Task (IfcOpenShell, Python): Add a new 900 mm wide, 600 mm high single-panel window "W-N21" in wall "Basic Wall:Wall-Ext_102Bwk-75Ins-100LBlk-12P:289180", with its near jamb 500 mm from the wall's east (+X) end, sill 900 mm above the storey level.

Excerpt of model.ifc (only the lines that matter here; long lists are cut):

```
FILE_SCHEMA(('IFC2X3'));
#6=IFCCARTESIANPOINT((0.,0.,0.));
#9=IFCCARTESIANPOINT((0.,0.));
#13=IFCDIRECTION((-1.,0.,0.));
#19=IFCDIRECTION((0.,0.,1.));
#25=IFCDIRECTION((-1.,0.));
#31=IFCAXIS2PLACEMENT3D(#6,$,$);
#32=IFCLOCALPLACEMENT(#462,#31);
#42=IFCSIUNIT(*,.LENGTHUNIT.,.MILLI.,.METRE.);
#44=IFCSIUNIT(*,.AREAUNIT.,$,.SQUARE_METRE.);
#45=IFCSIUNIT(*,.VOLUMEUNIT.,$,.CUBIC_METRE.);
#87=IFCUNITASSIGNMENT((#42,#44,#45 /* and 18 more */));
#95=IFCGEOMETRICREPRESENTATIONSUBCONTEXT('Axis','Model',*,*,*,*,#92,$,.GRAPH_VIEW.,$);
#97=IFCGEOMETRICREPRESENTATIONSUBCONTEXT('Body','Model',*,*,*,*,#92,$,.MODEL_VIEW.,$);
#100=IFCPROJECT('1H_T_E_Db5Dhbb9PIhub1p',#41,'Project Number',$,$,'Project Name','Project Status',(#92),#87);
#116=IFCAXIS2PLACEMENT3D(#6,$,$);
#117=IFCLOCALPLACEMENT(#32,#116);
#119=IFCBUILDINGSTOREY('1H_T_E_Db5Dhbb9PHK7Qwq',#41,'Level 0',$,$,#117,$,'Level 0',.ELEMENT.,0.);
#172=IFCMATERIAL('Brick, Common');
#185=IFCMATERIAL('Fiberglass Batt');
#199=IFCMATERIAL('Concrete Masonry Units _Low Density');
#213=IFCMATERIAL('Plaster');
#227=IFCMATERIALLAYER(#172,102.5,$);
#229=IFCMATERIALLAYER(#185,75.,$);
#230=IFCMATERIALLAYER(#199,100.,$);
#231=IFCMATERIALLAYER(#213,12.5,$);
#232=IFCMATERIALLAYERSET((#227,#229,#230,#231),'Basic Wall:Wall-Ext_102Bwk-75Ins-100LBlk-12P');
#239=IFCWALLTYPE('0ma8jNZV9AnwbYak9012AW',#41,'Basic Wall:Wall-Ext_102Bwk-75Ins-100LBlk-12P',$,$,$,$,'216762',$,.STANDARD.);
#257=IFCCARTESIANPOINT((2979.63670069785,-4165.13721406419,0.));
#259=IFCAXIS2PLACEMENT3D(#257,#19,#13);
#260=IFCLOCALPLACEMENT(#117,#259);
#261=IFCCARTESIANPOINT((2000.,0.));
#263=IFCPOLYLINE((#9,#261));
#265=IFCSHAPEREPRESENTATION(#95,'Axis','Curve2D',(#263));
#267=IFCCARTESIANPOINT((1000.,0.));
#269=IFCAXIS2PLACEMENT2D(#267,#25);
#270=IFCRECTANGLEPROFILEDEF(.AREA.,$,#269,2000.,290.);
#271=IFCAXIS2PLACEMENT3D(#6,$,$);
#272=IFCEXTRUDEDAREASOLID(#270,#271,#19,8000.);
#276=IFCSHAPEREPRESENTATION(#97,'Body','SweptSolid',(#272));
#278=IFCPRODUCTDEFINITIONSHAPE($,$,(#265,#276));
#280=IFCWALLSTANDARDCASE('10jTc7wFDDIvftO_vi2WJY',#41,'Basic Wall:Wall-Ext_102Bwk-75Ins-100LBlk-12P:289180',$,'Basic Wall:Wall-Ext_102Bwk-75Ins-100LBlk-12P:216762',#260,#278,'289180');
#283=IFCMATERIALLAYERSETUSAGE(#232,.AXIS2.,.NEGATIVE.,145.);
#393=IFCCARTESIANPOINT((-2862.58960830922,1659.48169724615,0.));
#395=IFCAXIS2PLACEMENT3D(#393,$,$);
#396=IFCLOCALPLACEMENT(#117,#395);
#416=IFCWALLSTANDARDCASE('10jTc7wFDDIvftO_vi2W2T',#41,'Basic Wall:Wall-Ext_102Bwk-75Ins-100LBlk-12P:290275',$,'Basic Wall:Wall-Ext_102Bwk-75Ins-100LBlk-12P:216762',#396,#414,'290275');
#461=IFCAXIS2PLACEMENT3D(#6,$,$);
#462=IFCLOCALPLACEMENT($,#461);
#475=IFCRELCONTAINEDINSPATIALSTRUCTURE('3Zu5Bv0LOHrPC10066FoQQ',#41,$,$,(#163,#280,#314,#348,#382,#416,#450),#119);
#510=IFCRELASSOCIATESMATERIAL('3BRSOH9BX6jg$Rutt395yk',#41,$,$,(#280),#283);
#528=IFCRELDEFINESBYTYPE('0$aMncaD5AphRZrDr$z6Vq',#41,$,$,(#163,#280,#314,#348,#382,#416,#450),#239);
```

```python
import numpy as np
import ifcopenshell
import ifcopenshell.api.feature
import ifcopenshell.api.geometry
import ifcopenshell.api.root
import ifcopenshell.api.spatial
import ifcopenshell.api.type
import ifcopenshell.geom
import ifcopenshell.util.element
import ifcopenshell.util.placement
import ifcopenshell.util.representation
import ifcopenshell.util.shape
import ifcopenshell.util.unit

model = ifcopenshell.open("model.ifc")
unit_scale = ifcopenshell.util.unit.calculate_unit_scale(model)
settings = ifcopenshell.geom.settings()


def volume(element):
    """Net volume in cubic metres, openings subtracted."""
    shape = ifcopenshell.geom.create_shape(settings, element)
    return ifcopenshell.util.shape.get_volume(shape.geometry)


wall = model.by_guid("10jTc7wFDDIvftO_vi2WJY")
storey = ifcopenshell.util.element.get_container(wall, ifc_class="IfcBuildingStorey")
context = ifcopenshell.util.representation.get_context(model, "Model", "Body", "MODEL_VIEW")
before = volume(wall)

width, height, from_end, sill = 0.9, 0.6, 0.5, 0.9  # metres

# The wall runs along its own X axis, and the end named is its -X end.
wall_shape = ifcopenshell.geom.create_shape(settings, wall)
x, y, z = ifcopenshell.util.shape.get_vertices(wall_shape.geometry).T
start = x.min() + from_end
face, thickness = float(y.min()), float(y.max() - y.min())
wall_matrix = ifcopenshell.util.placement.get_local_placement(wall.ObjectPlacement)
level = ifcopenshell.util.placement.get_local_placement(storey.ObjectPlacement)[2, 3]


def in_wall(x, y):
    """Placement at x, y metres in the wall's axes, at sill height."""
    matrix = wall_matrix.copy()
    matrix[:, 3] = wall_matrix @ np.array([x / unit_scale, y / unit_scale, 0.0, 1.0])
    matrix[2, 3] = level + sill / unit_scale
    return matrix


# Opening: a box that overshoots both wall faces by 50 mm.
opening = ifcopenshell.api.root.create_entity(model, ifc_class="IfcOpeningElement")
box = ifcopenshell.api.geometry.add_wall_representation(
    model, context=context, length=width, height=height, thickness=thickness + 0.1
)
ifcopenshell.api.geometry.assign_representation(model, product=opening, representation=box)
ifcopenshell.api.geometry.edit_object_placement(model, product=opening, matrix=in_wall(start, face - 0.05), is_si=False)
ifcopenshell.api.feature.add_feature(model, feature=opening, element=wall)

window = ifcopenshell.api.root.create_entity(model, ifc_class="IfcWindow", name="W-N21")
window.OverallWidth, window.OverallHeight = width / unit_scale, height / unit_scale
body = ifcopenshell.api.geometry.add_window_representation(
    model,
    context=context,
    overall_width=window.OverallWidth,
    overall_height=window.OverallHeight,
    partition_type="SINGLE_PANEL",
)
ifcopenshell.api.geometry.assign_representation(model, product=window, representation=body)
ifcopenshell.api.spatial.assign_container(model, products=[window], relating_structure=storey)
fills = ifcopenshell.api.feature.add_filling(model, opening=opening, element=window)
fills.OwnerHistory = window.OwnerHistory  # required in IFC2X3

# IFC2X3 keeps the operation on the window style.
style = ifcopenshell.api.root.create_entity(model, ifc_class="IfcWindowStyle", name="W-N21")
style.OperationType, style.ConstructionType = "SINGLE_PANEL", "NOTDEFINED"
style.ParameterTakesPrecedence = style.Sizeable = False
ifcopenshell.api.type.assign_type(model, related_objects=[window], relating_type=style)

# Centre the window in the wall's thickness.
ifcopenshell.api.geometry.edit_object_placement(model, product=window, matrix=in_wall(start, face), is_si=False)
window_shape = ifcopenshell.geom.create_shape(settings, window)
depth = ifcopenshell.util.shape.get_vertices(window_shape.geometry)[:, 1]
offset = face + thickness / 2 - (depth.min() + depth.max()) / 2
ifcopenshell.api.geometry.edit_object_placement(model, product=window, matrix=in_wall(start, offset), is_si=False)

after = volume(wall)

print(f"wall volume {before:.3f} -> {after:.3f} m3")

model.write("model_rev.ifc")
```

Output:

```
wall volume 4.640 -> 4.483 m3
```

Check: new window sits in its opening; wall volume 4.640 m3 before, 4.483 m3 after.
